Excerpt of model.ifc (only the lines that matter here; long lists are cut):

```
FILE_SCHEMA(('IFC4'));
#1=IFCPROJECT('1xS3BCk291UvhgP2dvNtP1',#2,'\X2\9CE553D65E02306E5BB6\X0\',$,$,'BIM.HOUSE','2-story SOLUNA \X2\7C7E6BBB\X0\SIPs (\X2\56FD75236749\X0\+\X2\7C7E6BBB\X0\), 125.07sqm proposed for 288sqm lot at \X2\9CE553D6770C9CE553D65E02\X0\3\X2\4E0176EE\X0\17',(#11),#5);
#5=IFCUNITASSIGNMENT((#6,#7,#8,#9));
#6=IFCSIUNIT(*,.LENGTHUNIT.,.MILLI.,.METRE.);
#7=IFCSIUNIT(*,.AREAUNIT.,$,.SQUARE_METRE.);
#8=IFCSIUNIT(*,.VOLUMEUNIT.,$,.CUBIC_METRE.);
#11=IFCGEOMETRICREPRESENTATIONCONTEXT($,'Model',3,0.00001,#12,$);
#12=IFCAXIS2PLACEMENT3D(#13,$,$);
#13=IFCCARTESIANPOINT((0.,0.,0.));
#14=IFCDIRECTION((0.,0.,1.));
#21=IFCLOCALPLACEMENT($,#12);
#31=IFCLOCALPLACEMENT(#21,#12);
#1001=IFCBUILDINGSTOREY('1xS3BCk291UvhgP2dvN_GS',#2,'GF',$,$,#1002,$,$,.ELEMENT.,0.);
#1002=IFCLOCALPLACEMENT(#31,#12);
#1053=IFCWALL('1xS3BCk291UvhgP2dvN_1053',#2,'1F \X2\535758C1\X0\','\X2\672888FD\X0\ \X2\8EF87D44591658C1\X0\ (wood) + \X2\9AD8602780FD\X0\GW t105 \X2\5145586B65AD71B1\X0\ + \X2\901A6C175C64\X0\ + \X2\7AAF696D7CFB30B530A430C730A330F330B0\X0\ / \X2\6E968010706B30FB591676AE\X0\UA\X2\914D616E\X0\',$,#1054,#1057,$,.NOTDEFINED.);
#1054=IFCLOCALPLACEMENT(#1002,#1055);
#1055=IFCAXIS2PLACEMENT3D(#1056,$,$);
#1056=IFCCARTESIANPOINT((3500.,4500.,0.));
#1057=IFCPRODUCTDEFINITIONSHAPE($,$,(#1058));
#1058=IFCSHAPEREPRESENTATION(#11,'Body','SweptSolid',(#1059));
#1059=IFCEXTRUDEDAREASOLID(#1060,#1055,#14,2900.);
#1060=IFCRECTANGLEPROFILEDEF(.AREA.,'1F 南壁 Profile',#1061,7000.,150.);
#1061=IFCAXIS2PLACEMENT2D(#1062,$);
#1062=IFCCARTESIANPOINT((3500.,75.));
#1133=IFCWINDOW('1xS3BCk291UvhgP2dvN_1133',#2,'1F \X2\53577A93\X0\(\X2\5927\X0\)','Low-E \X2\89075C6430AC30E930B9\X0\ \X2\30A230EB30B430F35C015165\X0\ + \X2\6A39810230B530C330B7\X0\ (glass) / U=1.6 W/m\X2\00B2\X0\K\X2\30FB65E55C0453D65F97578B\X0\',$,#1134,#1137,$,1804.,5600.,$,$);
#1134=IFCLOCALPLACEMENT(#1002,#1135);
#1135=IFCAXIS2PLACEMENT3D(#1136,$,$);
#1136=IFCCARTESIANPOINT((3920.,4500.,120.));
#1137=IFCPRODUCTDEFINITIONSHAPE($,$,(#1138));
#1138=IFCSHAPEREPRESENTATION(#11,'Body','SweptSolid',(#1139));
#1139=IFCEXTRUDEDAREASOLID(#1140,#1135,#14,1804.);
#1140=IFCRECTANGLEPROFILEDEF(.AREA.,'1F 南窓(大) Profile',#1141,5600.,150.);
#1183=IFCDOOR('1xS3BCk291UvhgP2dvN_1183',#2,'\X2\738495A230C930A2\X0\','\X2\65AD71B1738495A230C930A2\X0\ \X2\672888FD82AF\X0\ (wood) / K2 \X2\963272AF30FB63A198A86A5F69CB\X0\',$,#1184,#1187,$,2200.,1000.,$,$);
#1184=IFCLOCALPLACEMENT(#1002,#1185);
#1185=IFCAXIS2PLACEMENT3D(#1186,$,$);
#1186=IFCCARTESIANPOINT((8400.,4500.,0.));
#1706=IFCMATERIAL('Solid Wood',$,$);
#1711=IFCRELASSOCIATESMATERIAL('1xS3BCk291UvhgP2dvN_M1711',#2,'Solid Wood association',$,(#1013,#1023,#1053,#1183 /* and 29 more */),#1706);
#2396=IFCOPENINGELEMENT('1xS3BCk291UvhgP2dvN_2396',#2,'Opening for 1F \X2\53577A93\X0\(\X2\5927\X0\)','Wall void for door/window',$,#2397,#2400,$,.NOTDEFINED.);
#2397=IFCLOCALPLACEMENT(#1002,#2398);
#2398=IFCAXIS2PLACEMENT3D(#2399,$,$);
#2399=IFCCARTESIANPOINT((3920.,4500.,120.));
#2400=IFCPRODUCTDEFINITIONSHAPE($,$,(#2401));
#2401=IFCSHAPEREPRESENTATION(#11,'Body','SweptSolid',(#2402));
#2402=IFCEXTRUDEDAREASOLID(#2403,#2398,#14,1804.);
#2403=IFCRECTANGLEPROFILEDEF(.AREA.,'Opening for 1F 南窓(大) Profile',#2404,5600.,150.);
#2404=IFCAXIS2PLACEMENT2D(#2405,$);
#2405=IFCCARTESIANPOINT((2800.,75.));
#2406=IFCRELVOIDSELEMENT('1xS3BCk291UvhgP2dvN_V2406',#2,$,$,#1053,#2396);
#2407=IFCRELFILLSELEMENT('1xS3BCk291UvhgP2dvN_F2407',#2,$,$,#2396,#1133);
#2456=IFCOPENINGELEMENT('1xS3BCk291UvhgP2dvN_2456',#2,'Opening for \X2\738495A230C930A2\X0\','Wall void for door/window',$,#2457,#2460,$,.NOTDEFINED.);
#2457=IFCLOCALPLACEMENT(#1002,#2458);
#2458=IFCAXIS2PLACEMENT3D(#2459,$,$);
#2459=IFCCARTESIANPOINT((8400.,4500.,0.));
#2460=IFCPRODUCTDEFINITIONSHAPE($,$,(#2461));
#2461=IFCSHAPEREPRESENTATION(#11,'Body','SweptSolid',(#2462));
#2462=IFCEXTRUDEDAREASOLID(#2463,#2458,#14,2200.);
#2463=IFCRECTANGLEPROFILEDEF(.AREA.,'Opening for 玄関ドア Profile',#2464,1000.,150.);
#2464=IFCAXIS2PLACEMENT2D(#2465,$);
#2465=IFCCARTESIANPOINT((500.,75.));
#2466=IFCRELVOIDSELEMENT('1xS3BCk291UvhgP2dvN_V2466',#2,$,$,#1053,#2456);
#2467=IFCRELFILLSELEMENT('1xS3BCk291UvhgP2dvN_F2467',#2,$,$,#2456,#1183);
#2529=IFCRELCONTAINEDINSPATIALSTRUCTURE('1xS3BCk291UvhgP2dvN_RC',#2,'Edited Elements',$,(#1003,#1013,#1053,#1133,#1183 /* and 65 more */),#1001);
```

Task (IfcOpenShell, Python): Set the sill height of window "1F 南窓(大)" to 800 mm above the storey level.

```python
import numpy as np
import ifcopenshell
import ifcopenshell.api.geometry
import ifcopenshell.geom
import ifcopenshell.util.element
import ifcopenshell.util.placement
import ifcopenshell.util.shape
import ifcopenshell.util.unit

model = ifcopenshell.open("model.ifc")
unit_scale = ifcopenshell.util.unit.calculate_unit_scale(model)

window = model.by_guid("1xS3BCk291UvhgP2dvN_1133")
opening = window.FillsVoids[0].RelatingOpeningElement
storey = ifcopenshell.util.element.get_container(window, ifc_class="IfcBuildingStorey")
level = ifcopenshell.util.placement.get_local_placement(storey.ObjectPlacement)[2, 3]

# The opening's origin need not be at the sill, so measure its lowest point.
shape = ifcopenshell.geom.create_shape(ifcopenshell.geom.settings(), opening)
bottom = ifcopenshell.util.shape.get_shape_bottom_elevation(shape, shape.geometry) / unit_scale
dz = level + 0.8 / unit_scale - bottom

shift = np.array([0.0, 0.0, dz])
# The window is not placed relative to its opening, so move both.
for product in (opening, window):
    matrix = ifcopenshell.util.placement.get_local_placement(product.ObjectPlacement)
    matrix[:3, 3] += shift
    ifcopenshell.api.geometry.edit_object_placement(model, product=product, matrix=matrix, is_si=False)

print(f"moved by {dz * unit_scale:+.3f} m")

model.write("model_rev.ifc")
```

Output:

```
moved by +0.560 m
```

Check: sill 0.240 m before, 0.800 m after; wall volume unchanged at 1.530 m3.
